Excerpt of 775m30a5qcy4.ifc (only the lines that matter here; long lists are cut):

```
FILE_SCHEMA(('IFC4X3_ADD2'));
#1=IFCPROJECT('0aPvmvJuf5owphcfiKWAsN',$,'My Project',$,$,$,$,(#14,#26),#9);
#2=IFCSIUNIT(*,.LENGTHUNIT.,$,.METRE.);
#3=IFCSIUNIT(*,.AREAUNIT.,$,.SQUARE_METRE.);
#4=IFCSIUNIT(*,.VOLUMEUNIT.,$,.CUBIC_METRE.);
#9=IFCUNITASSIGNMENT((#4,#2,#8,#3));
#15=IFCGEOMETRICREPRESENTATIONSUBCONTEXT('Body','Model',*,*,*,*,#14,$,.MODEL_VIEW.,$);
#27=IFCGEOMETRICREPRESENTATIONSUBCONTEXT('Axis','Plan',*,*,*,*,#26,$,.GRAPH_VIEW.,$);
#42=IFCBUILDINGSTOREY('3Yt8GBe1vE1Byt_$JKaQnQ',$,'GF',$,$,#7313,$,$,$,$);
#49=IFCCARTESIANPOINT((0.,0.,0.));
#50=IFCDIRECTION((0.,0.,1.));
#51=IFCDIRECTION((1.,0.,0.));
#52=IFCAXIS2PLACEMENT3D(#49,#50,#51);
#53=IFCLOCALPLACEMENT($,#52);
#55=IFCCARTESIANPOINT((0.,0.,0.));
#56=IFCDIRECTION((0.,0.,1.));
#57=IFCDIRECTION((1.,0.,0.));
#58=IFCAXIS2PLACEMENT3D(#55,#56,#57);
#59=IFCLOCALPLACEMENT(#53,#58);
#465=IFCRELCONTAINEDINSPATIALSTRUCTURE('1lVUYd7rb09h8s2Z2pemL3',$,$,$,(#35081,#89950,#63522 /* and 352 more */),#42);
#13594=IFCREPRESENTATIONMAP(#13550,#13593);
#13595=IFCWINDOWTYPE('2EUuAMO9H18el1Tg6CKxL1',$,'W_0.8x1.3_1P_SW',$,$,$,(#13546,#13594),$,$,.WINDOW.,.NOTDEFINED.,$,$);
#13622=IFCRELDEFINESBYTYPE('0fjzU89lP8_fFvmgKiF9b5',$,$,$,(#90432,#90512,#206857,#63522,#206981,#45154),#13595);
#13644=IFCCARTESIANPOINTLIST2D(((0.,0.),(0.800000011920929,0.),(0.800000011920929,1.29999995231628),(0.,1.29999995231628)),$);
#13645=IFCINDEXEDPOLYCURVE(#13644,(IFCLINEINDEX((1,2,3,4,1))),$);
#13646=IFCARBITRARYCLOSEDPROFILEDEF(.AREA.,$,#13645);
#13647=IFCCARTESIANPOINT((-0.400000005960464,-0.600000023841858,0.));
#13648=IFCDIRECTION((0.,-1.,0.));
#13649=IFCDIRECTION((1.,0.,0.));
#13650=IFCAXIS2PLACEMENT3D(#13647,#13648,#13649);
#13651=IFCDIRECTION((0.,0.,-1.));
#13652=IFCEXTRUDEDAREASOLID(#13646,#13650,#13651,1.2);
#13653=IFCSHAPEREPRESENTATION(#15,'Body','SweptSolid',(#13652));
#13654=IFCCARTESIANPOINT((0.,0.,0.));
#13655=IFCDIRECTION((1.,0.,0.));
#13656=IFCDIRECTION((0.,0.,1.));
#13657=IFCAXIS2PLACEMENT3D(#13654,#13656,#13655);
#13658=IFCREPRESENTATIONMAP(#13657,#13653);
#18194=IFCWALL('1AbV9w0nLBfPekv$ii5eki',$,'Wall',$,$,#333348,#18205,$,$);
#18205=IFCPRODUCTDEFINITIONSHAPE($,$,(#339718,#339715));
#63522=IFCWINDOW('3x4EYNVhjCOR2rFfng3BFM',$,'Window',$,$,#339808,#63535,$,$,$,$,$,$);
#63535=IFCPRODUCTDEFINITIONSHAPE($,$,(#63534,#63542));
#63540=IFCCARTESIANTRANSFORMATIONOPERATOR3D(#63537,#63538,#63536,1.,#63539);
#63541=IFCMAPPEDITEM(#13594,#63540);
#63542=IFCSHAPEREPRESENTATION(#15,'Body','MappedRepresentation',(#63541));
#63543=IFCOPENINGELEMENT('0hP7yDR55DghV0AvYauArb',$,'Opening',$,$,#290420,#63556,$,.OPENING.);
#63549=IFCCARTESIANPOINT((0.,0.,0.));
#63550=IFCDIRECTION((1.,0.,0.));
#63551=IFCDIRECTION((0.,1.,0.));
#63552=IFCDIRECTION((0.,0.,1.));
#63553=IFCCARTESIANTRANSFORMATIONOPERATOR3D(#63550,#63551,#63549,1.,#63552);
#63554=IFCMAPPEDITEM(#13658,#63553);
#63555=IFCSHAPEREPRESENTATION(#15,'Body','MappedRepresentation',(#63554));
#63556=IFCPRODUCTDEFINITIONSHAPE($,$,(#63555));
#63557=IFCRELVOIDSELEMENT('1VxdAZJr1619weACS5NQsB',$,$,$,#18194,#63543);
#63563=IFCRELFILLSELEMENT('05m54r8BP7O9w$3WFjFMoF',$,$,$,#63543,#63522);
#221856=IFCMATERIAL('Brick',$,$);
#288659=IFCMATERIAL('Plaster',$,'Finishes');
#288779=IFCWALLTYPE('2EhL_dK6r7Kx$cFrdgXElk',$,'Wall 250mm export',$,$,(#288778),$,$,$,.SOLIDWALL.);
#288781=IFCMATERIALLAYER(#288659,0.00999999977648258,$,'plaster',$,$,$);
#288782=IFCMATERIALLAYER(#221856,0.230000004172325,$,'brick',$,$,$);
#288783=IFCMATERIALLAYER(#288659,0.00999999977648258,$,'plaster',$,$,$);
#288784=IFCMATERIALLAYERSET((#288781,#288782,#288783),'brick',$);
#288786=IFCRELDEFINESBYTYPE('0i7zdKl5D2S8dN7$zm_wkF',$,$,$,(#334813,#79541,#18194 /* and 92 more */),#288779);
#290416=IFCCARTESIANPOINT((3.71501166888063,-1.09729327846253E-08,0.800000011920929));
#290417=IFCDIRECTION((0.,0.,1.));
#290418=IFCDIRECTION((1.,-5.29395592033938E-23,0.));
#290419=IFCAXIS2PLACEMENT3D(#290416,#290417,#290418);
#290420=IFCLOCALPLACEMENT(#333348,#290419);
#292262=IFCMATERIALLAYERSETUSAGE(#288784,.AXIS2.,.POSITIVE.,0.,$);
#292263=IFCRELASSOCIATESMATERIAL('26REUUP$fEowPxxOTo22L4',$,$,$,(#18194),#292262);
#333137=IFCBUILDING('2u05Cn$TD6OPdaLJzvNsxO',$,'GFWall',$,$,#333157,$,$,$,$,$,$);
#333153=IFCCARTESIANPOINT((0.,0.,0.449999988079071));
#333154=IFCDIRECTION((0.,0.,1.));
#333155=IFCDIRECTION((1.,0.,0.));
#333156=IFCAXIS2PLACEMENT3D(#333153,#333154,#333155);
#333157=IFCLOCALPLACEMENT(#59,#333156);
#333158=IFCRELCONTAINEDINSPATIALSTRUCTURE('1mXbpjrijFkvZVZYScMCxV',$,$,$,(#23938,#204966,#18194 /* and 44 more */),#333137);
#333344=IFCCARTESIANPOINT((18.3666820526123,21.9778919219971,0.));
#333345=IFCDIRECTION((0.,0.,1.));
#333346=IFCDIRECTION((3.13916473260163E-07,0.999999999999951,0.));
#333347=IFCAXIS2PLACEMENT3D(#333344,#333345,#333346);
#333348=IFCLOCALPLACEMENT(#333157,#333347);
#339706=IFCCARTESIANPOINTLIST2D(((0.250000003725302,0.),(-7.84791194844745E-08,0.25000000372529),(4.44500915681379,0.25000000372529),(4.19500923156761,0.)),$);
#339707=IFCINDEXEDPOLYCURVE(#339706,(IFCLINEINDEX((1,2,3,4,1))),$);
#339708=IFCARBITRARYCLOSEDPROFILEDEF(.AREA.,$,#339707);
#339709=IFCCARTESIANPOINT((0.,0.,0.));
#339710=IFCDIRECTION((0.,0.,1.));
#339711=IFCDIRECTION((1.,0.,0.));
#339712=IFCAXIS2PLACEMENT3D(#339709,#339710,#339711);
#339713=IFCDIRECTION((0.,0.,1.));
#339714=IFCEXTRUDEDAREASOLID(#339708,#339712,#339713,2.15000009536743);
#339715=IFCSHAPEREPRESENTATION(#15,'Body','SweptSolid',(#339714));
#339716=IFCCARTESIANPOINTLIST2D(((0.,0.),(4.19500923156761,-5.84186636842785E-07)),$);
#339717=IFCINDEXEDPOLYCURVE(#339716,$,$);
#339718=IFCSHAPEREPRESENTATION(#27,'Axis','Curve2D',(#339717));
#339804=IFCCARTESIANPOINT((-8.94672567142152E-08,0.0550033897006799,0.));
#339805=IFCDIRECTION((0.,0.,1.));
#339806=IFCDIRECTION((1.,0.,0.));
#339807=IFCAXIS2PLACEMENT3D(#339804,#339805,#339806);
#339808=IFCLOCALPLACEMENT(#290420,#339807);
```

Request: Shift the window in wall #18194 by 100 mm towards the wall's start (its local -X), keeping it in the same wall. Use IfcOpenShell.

```python
import ifcopenshell
import ifcopenshell.api.geometry
import ifcopenshell.util.placement

model = ifcopenshell.open("775m30a5qcy4.ifc")

window = model.by_guid("3x4EYNVhjCOR2rFfng3BFM")
opening = window.FillsVoids[0].RelatingOpeningElement
wall = opening.VoidsElements[0].RelatingBuildingElement

wall_matrix = ifcopenshell.util.placement.get_local_placement(wall.ObjectPlacement)
shift = wall_matrix[:3, 0] * -0.1
before = ifcopenshell.util.placement.get_local_placement(window.ObjectPlacement)[:3, 3].copy()

# The window is placed relative to its opening, so it follows when the opening moves.
matrix = ifcopenshell.util.placement.get_local_placement(opening.ObjectPlacement)
matrix[:3, 3] += shift
ifcopenshell.api.geometry.edit_object_placement(
    model, product=opening, matrix=matrix, is_si=False, should_transform_children=True
)

after = ifcopenshell.util.placement.get_local_placement(window.ObjectPlacement)[:3, 3]
print("window moved by", (after - before).round(3) + 0.0)

model.write("775m30a5qcy4_rev.ifc")
```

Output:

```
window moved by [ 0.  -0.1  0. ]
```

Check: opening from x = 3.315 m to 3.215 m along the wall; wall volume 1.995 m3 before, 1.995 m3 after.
